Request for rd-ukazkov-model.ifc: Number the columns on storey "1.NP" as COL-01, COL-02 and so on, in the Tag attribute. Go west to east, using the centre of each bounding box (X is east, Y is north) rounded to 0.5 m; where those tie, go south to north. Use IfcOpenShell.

First a look at what the model holds.

```python
import ifcopenshell
import ifcopenshell.util.element
import ifcopenshell.util.placement

model = ifcopenshell.open("rd-ukazkov-model.ifc")
print(model.schema)
storey = next(s for s in model.by_type("IfcBuildingStorey") if s.Name == "1.NP")
columns = [e for e in ifcopenshell.util.element.get_decomposition(storey) if e.is_a("IfcColumn")]
for e in sorted(columns, key=lambda e: e.id()):
    origin = ifcopenshell.util.placement.get_local_placement(e.ObjectPlacement)[:3, 3]
    print(e.id(), e.Tag, e.Name, origin.round(2) + 0.0, sep=" | ")
```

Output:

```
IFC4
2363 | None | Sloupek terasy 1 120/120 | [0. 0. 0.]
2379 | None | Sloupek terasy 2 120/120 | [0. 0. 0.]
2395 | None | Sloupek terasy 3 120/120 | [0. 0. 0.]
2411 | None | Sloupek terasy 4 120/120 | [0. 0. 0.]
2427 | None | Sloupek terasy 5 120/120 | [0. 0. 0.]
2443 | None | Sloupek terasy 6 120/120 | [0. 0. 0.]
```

```python
import ifcopenshell
import ifcopenshell.geom
import ifcopenshell.util.element
import ifcopenshell.util.shape

model = ifcopenshell.open("rd-ukazkov-model.ifc")
settings = ifcopenshell.geom.settings()
settings.set("use-world-coords", True)


def centre(element):
    shape = ifcopenshell.geom.create_shape(settings, element)
    return ifcopenshell.util.shape.get_bbox_centroid(shape.geometry)


storey = next(s for s in model.by_type("IfcBuildingStorey") if s.Name == "1.NP")
columns = [e for e in ifcopenshell.util.element.get_decomposition(storey) if e.is_a("IfcColumn")]

# Insertion points can sit at a corner or the storey origin, so sort by the geometry (in metres).
centres = {e: centre(e) for e in columns}
columns.sort(key=lambda e: (round(centres[e][0] / 0.5), centres[e][1]))

for i, e in enumerate(columns, start=1):
    number = f"COL-{i:02d}"
    e.Tag = number
    print(e.id(), number)

model.write("rd-ukazkov-model_updated.ifc")
```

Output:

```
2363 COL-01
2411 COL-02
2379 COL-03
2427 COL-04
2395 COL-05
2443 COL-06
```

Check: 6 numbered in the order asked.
